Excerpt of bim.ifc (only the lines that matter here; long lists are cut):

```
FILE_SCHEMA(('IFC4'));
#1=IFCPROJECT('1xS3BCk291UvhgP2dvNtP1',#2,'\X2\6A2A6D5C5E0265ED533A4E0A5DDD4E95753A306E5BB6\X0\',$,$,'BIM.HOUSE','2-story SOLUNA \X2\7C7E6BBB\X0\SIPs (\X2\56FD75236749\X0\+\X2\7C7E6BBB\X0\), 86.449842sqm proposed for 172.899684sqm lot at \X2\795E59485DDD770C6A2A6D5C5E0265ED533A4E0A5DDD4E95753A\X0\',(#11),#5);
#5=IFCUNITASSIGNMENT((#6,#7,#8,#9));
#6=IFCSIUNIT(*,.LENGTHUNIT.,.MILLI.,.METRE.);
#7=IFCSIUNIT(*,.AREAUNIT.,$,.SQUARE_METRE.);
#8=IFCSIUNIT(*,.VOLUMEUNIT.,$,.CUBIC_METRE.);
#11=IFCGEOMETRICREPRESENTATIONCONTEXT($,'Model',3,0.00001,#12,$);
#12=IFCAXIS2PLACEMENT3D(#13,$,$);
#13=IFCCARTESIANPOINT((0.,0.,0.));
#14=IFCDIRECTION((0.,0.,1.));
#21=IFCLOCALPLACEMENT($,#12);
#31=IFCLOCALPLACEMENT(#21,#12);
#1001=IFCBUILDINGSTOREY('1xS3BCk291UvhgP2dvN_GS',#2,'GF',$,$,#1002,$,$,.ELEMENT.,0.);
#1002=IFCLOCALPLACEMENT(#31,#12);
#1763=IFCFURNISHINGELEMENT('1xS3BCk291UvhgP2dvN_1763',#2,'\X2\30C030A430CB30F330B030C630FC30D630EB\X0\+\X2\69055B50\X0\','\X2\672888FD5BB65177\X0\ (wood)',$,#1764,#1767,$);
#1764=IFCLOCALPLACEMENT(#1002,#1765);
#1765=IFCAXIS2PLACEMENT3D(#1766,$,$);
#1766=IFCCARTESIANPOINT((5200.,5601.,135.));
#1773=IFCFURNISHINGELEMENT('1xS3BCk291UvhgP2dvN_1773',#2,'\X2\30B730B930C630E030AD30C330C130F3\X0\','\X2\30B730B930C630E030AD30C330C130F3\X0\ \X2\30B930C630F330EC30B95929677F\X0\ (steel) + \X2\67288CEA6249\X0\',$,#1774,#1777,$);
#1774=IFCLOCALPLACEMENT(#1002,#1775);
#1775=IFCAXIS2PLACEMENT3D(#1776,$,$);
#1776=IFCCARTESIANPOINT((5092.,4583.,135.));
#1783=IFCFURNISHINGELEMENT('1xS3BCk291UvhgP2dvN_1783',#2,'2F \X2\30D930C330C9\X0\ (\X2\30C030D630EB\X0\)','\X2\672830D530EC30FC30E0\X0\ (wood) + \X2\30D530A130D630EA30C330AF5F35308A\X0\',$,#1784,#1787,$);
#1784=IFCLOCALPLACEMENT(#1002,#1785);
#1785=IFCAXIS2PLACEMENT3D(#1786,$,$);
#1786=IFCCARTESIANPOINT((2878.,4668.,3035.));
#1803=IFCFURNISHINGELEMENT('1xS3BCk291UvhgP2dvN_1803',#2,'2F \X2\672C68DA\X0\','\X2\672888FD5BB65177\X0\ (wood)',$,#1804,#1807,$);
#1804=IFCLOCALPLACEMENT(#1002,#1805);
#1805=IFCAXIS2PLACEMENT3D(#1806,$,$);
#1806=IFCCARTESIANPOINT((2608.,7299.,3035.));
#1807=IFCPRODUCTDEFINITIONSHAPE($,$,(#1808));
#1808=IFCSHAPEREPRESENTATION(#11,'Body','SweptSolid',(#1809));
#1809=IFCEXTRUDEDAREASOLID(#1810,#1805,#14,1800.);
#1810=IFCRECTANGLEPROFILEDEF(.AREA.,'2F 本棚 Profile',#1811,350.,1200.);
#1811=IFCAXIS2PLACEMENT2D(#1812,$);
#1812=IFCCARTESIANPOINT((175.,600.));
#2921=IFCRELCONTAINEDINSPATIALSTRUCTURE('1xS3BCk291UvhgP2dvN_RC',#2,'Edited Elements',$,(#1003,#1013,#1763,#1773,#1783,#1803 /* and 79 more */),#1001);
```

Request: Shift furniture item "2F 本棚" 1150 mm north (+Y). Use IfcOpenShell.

```python
import ifcopenshell
import ifcopenshell.api.geometry
import ifcopenshell.util.placement

model = ifcopenshell.open("bim.ifc")

item = model.by_guid("1xS3BCk291UvhgP2dvN_1803")
matrix = ifcopenshell.util.placement.get_local_placement(item.ObjectPlacement)
matrix[1, 3] += 1150.0
ifcopenshell.api.geometry.edit_object_placement(model, product=item, matrix=matrix, is_si=False)

print(ifcopenshell.util.placement.get_local_placement(item.ObjectPlacement).round(3) + 0.0)

model.write("bim-out.ifc")
```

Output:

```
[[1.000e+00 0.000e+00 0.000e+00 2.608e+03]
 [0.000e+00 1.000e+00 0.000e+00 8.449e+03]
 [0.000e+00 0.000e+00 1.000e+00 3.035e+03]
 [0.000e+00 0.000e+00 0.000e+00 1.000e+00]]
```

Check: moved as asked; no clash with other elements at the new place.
